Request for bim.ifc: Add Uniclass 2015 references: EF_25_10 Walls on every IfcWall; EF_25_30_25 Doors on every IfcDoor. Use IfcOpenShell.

First a look at what the model holds.

```python
import ifcopenshell

model = ifcopenshell.open("bim.ifc")
print(model.schema)
print("classifications:", [c.Name for c in model.by_type("IfcClassification")])
for ifc_class in ("IfcDoor", "IfcRoof", "IfcStair", "IfcWall", "IfcWindow"):
    print(ifc_class, len(model.by_type(ifc_class)))
```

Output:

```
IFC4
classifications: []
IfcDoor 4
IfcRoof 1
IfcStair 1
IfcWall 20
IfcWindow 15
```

```python
import ifcopenshell
import ifcopenshell.api.classification

model = ifcopenshell.open("bim.ifc")

system = ifcopenshell.api.classification.add_classification(model, classification="Uniclass 2015")

codes = {
    "IfcWall": ("EF_25_10", "Walls"),
    "IfcDoor": ("EF_25_30_25", "Doors"),
}
for ifc_class, (code, name) in codes.items():
    products = model.by_type(ifc_class)
    ifcopenshell.api.classification.add_reference(
        model, products=products, classification=system, identification=code, name=name
    )
    print(code, len(products))

model.write("bim_rev.ifc")
```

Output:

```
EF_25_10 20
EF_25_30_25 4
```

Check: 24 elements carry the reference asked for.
